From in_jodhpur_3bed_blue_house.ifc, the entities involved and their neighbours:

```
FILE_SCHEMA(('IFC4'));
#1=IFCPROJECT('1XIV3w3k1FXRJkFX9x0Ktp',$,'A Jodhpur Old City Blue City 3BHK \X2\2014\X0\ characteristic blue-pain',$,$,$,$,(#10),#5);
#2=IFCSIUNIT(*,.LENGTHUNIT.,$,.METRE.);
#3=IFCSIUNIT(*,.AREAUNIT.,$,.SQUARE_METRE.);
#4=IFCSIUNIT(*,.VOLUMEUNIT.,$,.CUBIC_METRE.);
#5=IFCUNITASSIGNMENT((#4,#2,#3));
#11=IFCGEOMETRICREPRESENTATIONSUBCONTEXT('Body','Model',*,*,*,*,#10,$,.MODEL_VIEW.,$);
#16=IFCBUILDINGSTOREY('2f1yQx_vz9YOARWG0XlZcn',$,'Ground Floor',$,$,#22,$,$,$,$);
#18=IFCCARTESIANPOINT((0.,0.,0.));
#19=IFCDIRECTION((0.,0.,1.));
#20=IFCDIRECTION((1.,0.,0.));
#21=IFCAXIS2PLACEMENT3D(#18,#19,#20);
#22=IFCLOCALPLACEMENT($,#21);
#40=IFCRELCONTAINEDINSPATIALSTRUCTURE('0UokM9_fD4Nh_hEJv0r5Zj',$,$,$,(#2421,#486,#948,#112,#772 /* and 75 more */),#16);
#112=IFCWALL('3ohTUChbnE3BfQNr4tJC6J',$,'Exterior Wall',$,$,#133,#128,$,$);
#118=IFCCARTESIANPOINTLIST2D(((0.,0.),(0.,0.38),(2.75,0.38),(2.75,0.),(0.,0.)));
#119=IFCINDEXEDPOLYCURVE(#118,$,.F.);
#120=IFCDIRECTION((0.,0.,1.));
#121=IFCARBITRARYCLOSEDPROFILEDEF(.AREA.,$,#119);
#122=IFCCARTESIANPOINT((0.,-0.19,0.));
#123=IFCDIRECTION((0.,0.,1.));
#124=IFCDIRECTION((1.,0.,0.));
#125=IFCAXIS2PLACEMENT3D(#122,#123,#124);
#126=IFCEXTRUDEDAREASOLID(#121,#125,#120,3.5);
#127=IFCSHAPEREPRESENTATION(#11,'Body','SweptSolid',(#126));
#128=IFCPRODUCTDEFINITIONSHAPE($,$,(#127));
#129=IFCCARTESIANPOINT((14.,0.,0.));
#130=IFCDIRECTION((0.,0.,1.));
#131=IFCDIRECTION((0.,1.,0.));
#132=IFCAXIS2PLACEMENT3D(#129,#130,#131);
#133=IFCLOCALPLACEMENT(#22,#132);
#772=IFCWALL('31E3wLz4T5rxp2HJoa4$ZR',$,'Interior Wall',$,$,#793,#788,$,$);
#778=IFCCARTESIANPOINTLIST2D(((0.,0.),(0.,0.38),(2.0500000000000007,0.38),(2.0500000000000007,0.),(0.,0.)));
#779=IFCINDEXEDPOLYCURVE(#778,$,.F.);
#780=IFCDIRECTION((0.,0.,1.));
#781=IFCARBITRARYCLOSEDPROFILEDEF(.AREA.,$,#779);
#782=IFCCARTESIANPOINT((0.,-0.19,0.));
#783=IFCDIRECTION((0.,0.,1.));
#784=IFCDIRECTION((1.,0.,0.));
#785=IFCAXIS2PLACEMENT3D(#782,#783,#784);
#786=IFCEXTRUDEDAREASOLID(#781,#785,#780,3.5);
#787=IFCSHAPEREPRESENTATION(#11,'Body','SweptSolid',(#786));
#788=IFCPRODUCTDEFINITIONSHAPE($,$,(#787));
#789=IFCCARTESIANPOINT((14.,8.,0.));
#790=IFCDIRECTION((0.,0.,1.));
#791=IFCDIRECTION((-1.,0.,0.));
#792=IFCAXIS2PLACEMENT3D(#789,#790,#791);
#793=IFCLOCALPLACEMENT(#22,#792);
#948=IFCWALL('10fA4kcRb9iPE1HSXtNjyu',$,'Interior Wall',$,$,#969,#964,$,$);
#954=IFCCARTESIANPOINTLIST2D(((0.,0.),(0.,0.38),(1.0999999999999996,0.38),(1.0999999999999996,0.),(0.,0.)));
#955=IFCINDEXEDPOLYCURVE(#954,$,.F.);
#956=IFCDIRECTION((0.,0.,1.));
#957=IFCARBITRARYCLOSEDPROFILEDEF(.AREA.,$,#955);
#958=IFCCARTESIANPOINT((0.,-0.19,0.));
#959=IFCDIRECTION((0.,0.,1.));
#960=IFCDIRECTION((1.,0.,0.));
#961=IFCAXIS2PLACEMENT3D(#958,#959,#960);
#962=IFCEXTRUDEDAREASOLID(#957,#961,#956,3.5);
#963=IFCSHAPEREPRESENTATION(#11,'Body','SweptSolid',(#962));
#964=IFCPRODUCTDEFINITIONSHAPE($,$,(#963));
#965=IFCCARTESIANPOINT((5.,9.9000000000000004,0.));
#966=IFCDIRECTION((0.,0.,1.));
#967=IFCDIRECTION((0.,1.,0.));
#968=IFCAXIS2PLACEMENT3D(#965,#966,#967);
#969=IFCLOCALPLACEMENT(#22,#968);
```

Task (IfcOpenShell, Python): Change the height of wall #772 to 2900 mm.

```python
import ifcopenshell
import ifcopenshell.geom
import ifcopenshell.util.representation
import ifcopenshell.util.shape
import ifcopenshell.util.unit

model = ifcopenshell.open("in_jodhpur_3bed_blue_house.ifc")
unit_scale = ifcopenshell.util.unit.calculate_unit_scale(model)
settings = ifcopenshell.geom.settings()


def volume(element):
    """Net volume in cubic metres, openings subtracted."""
    shape = ifcopenshell.geom.create_shape(settings, element)
    return ifcopenshell.util.shape.get_volume(shape.geometry)


wall = model.by_guid("31E3wLz4T5rxp2HJoa4$ZR")
before = volume(wall)

body = ifcopenshell.util.representation.get_representation(wall, "Model", "Body")
solid = body.Items[0]
old_height = solid.Depth
solid.Depth = 2.9 / unit_scale
after = volume(wall)

print(f"height {old_height:g} -> {solid.Depth:g}, volume {before:.3f} -> {after:.3f} m3")

model.write("in_jodhpur_3bed_blue_house_edited.ifc")
```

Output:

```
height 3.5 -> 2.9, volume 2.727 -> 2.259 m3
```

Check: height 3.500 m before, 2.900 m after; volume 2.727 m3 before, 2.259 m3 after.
